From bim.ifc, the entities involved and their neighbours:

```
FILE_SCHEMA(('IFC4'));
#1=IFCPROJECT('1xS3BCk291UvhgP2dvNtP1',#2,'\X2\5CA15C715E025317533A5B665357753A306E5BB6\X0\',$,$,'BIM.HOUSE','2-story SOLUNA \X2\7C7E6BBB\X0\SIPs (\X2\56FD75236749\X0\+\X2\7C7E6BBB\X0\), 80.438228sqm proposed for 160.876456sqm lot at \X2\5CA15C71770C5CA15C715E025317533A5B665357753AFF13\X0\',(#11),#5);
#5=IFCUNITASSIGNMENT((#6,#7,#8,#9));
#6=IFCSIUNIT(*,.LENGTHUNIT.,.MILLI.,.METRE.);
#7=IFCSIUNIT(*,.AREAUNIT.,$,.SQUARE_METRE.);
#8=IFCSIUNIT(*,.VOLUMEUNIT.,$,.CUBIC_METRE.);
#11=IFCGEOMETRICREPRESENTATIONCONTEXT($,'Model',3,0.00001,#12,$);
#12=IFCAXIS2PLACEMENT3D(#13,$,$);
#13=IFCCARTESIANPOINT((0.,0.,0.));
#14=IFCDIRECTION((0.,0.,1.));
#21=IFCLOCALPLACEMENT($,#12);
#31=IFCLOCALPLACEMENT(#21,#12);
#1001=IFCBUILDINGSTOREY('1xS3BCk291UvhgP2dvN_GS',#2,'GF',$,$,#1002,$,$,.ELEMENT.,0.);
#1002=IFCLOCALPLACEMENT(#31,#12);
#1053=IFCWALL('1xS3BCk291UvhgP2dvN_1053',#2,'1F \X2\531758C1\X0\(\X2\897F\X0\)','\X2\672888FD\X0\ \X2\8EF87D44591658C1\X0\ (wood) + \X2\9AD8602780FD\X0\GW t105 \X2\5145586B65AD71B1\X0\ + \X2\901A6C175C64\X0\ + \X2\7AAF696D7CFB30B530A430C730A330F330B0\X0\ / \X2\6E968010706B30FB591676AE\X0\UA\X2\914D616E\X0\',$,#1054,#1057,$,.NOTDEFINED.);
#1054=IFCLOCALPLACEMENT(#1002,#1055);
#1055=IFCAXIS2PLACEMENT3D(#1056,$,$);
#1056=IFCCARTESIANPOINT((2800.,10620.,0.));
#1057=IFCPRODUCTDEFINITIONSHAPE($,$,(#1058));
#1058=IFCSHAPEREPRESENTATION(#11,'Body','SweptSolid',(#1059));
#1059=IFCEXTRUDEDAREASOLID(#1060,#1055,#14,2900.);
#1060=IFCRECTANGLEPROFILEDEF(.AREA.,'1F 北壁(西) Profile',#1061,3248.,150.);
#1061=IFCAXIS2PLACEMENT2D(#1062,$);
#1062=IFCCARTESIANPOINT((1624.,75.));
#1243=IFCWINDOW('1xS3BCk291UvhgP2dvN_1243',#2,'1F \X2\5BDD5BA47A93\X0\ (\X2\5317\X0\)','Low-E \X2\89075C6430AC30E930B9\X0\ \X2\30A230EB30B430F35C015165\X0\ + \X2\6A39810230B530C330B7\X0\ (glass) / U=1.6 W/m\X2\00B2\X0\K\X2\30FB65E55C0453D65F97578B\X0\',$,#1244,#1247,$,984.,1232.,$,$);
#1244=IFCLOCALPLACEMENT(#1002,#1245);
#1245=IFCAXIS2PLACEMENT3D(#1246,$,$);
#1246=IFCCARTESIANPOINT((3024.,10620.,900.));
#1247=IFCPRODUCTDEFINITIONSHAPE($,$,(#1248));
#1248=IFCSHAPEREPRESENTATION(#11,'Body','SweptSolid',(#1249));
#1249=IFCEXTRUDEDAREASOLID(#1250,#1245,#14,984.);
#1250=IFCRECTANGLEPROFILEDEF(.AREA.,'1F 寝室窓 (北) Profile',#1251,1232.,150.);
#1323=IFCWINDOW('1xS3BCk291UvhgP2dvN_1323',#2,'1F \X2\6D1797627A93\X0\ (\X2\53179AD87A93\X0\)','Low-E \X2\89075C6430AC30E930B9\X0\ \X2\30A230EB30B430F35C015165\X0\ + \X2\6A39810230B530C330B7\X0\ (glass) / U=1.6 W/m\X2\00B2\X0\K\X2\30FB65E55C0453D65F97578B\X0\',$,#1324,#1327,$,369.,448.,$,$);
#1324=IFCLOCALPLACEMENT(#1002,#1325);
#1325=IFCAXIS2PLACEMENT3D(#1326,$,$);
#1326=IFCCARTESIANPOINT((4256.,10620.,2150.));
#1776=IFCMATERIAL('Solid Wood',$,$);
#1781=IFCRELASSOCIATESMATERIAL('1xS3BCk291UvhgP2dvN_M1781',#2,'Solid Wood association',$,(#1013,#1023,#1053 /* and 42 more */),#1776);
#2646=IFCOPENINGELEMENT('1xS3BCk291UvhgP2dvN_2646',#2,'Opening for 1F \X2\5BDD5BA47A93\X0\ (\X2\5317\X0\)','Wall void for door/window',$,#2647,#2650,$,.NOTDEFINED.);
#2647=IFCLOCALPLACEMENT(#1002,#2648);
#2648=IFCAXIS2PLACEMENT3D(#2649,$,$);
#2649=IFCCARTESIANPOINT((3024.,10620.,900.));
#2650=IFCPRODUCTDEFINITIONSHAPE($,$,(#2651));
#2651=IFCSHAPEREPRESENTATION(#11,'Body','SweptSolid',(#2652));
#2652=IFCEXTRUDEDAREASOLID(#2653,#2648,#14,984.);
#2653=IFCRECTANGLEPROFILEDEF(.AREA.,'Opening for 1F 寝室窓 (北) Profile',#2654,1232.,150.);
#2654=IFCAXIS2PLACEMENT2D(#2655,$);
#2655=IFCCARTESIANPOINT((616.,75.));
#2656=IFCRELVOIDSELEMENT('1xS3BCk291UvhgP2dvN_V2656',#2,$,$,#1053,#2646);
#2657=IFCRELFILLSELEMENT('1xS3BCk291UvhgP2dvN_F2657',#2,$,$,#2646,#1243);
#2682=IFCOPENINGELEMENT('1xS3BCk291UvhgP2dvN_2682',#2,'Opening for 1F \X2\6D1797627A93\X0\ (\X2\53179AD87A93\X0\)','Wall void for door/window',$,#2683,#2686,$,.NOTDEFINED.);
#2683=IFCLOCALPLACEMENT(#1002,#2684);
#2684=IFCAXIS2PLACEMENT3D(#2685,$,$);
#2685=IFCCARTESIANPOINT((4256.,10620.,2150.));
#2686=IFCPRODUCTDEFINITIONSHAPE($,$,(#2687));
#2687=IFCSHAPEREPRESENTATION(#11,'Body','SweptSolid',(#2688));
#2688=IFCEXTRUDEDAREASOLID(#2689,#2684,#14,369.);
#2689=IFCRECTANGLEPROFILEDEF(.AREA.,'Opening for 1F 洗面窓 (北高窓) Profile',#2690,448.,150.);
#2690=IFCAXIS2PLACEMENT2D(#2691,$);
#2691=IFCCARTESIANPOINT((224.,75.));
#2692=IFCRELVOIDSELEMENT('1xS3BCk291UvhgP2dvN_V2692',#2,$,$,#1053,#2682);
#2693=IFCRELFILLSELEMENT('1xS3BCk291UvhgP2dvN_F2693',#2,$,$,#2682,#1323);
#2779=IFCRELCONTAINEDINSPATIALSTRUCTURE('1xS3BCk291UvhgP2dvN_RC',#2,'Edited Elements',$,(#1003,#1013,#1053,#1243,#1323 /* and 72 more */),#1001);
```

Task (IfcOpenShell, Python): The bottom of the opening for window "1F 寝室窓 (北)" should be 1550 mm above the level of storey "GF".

```python
import numpy as np
import ifcopenshell
import ifcopenshell.api.geometry
import ifcopenshell.geom
import ifcopenshell.util.element
import ifcopenshell.util.placement
import ifcopenshell.util.shape
import ifcopenshell.util.unit

model = ifcopenshell.open("bim.ifc")
unit_scale = ifcopenshell.util.unit.calculate_unit_scale(model)

window = model.by_guid("1xS3BCk291UvhgP2dvN_1243")
opening = window.FillsVoids[0].RelatingOpeningElement
storey = ifcopenshell.util.element.get_container(window, ifc_class="IfcBuildingStorey")
level = ifcopenshell.util.placement.get_local_placement(storey.ObjectPlacement)[2, 3]

# The opening's origin need not be at the sill, so measure its lowest point.
shape = ifcopenshell.geom.create_shape(ifcopenshell.geom.settings(), opening)
bottom = ifcopenshell.util.shape.get_shape_bottom_elevation(shape, shape.geometry) / unit_scale
dz = level + 1.55 / unit_scale - bottom

shift = np.array([0.0, 0.0, dz])
# The window is not placed relative to its opening, so move both.
for product in (opening, window):
    matrix = ifcopenshell.util.placement.get_local_placement(product.ObjectPlacement)
    matrix[:3, 3] += shift
    ifcopenshell.api.geometry.edit_object_placement(model, product=product, matrix=matrix, is_si=False)

print(f"moved by {dz * unit_scale:+.3f} m")

model.write("bim_v2.ifc")
```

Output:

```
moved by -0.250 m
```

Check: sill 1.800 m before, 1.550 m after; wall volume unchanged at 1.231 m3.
